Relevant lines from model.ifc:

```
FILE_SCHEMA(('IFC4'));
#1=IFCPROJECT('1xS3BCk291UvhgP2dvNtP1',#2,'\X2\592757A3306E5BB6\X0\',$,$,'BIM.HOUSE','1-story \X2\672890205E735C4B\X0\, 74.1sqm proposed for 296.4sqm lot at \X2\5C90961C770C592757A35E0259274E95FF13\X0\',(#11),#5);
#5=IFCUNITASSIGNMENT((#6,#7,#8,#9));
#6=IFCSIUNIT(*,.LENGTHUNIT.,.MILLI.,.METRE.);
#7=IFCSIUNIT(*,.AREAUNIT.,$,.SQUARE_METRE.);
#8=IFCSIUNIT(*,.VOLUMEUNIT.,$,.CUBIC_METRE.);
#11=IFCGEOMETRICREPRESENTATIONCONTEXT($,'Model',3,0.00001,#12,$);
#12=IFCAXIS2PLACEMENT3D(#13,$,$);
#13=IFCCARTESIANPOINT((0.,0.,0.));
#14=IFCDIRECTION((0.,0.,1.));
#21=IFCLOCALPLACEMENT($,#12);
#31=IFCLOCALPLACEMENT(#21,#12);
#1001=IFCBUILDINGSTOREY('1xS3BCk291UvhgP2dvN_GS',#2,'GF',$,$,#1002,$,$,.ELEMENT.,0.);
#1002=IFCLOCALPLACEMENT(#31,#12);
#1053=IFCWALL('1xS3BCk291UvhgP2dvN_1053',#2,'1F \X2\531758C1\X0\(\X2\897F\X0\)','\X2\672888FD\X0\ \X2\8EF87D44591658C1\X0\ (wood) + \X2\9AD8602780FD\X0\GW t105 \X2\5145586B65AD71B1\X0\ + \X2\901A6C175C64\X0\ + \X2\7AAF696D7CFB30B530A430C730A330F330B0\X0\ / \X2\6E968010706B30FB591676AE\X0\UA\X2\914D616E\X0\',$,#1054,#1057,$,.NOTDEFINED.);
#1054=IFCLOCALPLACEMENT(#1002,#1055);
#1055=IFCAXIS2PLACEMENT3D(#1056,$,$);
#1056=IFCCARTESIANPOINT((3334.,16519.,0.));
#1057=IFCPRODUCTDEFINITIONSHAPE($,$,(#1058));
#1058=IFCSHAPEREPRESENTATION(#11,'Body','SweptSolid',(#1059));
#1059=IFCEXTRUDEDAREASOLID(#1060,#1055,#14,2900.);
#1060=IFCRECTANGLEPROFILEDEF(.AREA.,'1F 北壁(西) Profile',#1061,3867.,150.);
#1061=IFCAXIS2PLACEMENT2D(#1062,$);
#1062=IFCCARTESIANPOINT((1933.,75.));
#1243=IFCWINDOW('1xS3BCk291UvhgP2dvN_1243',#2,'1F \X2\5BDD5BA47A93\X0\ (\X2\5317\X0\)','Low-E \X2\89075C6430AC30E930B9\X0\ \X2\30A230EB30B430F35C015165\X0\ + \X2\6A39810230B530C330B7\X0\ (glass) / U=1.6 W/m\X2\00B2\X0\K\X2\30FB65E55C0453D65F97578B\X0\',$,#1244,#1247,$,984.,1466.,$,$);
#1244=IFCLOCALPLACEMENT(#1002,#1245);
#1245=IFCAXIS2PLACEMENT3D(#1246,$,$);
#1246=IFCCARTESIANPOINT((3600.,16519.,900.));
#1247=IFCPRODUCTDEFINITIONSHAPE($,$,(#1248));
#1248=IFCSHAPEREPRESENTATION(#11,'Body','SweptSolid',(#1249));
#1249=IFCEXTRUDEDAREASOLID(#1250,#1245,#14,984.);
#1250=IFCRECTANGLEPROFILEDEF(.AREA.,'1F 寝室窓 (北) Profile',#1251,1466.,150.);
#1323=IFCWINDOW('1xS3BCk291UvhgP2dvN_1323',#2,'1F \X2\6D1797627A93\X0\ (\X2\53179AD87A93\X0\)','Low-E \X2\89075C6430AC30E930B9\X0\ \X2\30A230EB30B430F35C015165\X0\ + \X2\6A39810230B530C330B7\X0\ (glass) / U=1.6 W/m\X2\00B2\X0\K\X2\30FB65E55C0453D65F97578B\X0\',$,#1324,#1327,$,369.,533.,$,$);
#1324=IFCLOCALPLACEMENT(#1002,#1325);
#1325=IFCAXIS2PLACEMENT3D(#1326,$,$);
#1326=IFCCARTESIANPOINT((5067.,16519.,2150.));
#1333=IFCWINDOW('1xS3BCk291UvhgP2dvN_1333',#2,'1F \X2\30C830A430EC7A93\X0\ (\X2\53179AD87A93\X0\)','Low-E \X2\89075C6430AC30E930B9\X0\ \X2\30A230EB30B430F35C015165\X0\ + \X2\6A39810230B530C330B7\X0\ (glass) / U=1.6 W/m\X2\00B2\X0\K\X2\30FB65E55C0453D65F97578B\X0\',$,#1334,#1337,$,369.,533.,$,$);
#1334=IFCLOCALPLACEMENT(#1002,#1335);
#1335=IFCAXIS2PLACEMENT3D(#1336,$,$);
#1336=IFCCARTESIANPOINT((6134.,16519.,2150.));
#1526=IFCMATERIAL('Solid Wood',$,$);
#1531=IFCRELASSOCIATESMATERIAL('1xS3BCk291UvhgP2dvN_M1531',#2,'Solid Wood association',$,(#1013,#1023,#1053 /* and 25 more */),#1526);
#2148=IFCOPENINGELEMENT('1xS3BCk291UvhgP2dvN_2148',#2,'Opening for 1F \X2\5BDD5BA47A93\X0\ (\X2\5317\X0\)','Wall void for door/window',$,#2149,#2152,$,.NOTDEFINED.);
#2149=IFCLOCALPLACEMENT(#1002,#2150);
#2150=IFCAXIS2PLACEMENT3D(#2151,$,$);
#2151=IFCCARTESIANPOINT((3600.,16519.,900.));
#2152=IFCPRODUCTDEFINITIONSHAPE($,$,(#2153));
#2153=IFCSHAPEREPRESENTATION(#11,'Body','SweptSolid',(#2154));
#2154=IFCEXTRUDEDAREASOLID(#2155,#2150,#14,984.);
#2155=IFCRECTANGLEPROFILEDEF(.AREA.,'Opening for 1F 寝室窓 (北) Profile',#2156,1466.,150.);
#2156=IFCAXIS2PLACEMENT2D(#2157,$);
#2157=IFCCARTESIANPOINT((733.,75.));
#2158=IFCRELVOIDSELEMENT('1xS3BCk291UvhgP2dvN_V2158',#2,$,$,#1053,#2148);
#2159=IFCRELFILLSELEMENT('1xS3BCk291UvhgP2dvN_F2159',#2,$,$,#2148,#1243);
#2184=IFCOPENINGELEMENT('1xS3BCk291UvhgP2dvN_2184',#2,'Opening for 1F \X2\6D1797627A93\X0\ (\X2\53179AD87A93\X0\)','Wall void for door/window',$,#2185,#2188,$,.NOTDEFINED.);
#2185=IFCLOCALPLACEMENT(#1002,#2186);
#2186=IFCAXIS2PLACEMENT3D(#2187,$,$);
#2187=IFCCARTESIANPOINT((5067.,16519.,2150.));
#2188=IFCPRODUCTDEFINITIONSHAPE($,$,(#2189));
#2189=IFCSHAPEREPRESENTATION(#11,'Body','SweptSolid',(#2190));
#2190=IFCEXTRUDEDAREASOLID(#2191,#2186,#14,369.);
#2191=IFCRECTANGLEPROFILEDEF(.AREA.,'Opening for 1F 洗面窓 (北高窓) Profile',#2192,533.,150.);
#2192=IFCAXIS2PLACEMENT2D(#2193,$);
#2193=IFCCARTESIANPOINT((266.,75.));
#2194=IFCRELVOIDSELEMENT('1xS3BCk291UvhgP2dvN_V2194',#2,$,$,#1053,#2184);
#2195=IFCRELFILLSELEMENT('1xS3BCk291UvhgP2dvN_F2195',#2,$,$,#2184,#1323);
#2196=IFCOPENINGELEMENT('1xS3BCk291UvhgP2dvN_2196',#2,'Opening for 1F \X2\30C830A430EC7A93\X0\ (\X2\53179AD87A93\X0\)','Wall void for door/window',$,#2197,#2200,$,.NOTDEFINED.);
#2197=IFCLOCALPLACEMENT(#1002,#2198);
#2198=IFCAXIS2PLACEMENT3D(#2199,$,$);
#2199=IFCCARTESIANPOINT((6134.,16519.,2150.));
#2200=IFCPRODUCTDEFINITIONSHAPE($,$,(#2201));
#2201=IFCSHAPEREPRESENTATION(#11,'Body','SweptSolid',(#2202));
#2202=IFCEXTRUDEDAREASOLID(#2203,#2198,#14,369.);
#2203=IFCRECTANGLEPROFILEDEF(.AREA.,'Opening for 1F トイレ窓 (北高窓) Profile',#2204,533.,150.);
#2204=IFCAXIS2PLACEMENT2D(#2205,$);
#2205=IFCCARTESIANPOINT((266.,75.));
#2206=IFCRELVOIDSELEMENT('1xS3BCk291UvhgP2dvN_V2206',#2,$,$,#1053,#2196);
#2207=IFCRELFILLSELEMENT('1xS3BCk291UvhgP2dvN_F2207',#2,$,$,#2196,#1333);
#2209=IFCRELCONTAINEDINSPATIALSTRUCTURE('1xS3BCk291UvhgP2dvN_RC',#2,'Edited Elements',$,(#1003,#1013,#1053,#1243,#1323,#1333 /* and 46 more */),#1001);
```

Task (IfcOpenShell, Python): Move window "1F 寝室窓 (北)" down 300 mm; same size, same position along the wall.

```python
import numpy as np
import ifcopenshell
import ifcopenshell.api.geometry
import ifcopenshell.util.placement
import ifcopenshell.util.unit

model = ifcopenshell.open("model.ifc")
unit_scale = ifcopenshell.util.unit.calculate_unit_scale(model)

window = model.by_id(1243)
opening = window.FillsVoids[0].RelatingOpeningElement
dz = -300.0

shift = np.array([0.0, 0.0, dz])
# The window is not placed relative to its opening, so move both.
for product in (opening, window):
    matrix = ifcopenshell.util.placement.get_local_placement(product.ObjectPlacement)
    matrix[:3, 3] += shift
    ifcopenshell.api.geometry.edit_object_placement(model, product=product, matrix=matrix, is_si=False)

print(f"moved by {dz * unit_scale:+.3f} m")

model.write("model-out.ifc")
```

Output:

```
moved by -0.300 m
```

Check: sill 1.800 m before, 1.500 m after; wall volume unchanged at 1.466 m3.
